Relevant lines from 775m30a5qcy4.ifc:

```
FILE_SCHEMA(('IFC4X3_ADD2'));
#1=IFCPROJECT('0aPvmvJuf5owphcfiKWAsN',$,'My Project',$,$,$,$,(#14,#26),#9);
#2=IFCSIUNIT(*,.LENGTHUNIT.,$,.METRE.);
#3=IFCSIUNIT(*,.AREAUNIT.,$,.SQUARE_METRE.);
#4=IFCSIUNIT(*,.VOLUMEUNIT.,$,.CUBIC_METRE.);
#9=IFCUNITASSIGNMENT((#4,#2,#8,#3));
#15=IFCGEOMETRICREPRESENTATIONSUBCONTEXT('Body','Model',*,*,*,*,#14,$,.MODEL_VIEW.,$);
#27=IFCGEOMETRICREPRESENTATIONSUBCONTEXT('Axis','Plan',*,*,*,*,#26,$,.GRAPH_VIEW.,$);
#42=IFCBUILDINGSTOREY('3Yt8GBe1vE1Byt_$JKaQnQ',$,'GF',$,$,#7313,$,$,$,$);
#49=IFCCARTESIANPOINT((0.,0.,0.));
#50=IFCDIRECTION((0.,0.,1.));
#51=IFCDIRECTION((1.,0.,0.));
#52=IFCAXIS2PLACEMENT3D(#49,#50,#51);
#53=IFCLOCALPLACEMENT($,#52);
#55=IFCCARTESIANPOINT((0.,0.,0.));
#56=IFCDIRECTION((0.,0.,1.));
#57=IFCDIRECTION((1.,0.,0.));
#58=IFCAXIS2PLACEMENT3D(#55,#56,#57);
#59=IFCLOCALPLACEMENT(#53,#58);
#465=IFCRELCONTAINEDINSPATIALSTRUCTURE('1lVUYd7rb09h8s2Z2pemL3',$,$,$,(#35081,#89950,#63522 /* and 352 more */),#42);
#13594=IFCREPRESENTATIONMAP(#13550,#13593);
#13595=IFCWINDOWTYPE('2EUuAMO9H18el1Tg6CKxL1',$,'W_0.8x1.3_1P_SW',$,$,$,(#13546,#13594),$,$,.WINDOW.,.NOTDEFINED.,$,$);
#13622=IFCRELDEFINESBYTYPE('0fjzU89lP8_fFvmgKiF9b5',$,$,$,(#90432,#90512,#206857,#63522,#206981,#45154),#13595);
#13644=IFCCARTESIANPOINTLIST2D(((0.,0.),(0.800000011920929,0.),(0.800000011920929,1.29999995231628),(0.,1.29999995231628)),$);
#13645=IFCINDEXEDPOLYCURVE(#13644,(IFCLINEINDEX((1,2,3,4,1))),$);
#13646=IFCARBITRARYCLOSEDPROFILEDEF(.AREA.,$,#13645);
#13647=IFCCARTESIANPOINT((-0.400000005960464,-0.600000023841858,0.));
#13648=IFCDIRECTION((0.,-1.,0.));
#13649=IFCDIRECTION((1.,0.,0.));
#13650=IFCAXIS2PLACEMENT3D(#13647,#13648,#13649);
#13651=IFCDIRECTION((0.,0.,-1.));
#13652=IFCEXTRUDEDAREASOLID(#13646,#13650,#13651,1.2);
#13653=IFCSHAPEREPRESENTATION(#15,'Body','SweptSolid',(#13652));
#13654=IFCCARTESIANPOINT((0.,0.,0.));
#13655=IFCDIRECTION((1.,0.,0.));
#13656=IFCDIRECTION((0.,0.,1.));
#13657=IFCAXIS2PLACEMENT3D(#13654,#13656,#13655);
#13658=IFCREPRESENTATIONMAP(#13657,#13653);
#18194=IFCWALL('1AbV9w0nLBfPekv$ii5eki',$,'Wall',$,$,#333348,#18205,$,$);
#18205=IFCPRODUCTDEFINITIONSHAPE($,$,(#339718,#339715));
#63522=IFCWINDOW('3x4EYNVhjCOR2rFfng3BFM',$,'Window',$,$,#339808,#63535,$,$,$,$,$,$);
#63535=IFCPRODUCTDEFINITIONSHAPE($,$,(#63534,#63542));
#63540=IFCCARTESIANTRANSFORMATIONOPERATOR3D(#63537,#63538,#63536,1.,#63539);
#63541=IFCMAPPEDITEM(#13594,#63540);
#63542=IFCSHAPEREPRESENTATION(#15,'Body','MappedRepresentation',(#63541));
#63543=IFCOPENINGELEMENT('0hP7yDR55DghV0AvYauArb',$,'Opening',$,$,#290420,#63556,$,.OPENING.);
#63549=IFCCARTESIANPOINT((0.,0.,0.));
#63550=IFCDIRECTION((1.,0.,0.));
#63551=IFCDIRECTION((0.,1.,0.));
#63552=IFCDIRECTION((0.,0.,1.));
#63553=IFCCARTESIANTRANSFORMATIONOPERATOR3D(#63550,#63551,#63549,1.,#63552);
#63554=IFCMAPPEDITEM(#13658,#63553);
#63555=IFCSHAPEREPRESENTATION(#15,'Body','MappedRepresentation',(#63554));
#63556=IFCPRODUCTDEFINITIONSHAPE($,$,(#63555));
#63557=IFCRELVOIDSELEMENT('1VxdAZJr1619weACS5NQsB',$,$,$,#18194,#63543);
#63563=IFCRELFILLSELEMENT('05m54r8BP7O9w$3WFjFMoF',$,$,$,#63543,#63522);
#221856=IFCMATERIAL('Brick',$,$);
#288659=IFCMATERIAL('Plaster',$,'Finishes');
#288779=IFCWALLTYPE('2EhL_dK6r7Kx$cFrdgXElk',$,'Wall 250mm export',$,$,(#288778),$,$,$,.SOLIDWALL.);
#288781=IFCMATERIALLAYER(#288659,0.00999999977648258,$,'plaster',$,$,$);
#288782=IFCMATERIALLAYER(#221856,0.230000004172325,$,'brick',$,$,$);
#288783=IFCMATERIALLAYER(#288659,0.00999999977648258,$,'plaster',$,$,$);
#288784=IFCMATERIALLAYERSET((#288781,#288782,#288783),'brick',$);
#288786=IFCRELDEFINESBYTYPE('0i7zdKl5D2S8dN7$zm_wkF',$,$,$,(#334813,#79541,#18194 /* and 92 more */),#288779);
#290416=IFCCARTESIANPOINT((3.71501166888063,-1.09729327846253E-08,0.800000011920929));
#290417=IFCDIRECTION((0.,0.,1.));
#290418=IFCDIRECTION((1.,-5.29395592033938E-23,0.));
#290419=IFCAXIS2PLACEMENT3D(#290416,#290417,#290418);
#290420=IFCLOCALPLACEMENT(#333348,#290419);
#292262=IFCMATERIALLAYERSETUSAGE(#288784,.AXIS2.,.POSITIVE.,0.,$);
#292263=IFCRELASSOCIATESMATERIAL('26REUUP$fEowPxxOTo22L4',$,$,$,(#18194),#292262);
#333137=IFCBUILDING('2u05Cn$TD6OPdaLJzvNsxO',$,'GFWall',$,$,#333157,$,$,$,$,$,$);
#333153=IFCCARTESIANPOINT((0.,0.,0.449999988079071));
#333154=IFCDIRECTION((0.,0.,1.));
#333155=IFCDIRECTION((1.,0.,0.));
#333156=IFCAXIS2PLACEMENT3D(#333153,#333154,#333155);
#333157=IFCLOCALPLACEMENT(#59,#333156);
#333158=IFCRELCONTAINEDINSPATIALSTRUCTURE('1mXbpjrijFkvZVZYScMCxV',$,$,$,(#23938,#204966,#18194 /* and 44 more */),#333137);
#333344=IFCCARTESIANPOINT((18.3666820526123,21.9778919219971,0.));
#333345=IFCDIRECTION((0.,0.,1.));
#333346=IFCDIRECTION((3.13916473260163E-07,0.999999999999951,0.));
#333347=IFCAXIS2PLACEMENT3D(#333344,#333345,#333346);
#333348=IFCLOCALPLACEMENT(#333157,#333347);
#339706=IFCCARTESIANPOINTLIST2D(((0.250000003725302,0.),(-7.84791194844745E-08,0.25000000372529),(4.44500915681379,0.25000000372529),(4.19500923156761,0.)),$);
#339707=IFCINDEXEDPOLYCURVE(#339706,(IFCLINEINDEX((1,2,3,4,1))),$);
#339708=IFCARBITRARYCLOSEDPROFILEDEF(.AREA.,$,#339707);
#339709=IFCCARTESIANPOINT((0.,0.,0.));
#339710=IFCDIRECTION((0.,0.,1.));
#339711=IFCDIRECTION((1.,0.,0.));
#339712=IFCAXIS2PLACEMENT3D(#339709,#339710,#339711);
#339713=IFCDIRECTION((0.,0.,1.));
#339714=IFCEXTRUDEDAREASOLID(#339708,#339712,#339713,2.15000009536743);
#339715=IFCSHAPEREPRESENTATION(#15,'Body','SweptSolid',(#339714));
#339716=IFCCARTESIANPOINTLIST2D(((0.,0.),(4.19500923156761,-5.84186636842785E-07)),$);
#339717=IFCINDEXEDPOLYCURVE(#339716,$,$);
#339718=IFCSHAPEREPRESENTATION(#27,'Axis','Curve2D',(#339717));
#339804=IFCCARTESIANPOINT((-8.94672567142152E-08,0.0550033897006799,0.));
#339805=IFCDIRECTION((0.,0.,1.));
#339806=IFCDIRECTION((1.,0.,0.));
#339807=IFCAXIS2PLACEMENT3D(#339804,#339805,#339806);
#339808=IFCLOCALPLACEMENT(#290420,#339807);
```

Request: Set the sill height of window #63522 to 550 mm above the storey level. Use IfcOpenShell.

```python
import numpy as np
import ifcopenshell
import ifcopenshell.api.geometry
import ifcopenshell.geom
import ifcopenshell.util.element
import ifcopenshell.util.placement
import ifcopenshell.util.shape
import ifcopenshell.util.unit

model = ifcopenshell.open("775m30a5qcy4.ifc")
unit_scale = ifcopenshell.util.unit.calculate_unit_scale(model)

window = model.by_guid("3x4EYNVhjCOR2rFfng3BFM")
opening = window.FillsVoids[0].RelatingOpeningElement
storey = ifcopenshell.util.element.get_container(window, ifc_class="IfcBuildingStorey")
level = ifcopenshell.util.placement.get_local_placement(storey.ObjectPlacement)[2, 3]

# The opening's origin need not be at the sill, so measure its lowest point.
shape = ifcopenshell.geom.create_shape(ifcopenshell.geom.settings(), opening)
bottom = ifcopenshell.util.shape.get_shape_bottom_elevation(shape, shape.geometry) / unit_scale
dz = level + 0.55 - bottom

shift = np.array([0.0, 0.0, dz])
# The window is placed relative to its opening, so it follows when the opening moves.
matrix = ifcopenshell.util.placement.get_local_placement(opening.ObjectPlacement)
matrix[:3, 3] += shift
ifcopenshell.api.geometry.edit_object_placement(
    model, product=opening, matrix=matrix, is_si=False, should_transform_children=True
)

print(f"moved by {dz * unit_scale:+.3f} m")

model.write("775m30a5qcy4_v2.ifc")
```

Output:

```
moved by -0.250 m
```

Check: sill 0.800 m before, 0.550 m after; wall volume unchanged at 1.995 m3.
